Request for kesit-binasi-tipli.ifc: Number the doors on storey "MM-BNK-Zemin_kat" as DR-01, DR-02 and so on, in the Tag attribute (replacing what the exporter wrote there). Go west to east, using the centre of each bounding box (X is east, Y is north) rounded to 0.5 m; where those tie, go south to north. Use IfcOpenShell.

First a look at what the model holds.

```python
import ifcopenshell
import ifcopenshell.util.element
import ifcopenshell.util.placement

model = ifcopenshell.open("kesit-binasi-tipli.ifc")
print(model.schema)
storey = next(s for s in model.by_type("IfcBuildingStorey") if s.Name == "MM-BNK-Zemin_kat")
doors = [e for e in ifcopenshell.util.element.get_decomposition(storey) if e.is_a("IfcDoor")]
for e in sorted(doors, key=lambda e: e.id()):
    origin = ifcopenshell.util.placement.get_local_placement(e.ObjectPlacement)[:3, 3]
    print(e.id(), e.Tag, e.Name, origin.round(2) + 0.0, sep=" | ")
```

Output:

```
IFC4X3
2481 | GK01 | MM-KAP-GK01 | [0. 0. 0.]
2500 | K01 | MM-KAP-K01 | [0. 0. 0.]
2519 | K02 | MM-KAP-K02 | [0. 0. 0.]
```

```python
import ifcopenshell
import ifcopenshell.geom
import ifcopenshell.util.element
import ifcopenshell.util.shape

model = ifcopenshell.open("kesit-binasi-tipli.ifc")
settings = ifcopenshell.geom.settings()
settings.set("use-world-coords", True)


def centre(element):
    shape = ifcopenshell.geom.create_shape(settings, element)
    return ifcopenshell.util.shape.get_bbox_centroid(shape.geometry)


storey = next(s for s in model.by_type("IfcBuildingStorey") if s.Name == "MM-BNK-Zemin_kat")
doors = [e for e in ifcopenshell.util.element.get_decomposition(storey) if e.is_a("IfcDoor")]

# Insertion points can sit at a corner or the storey origin, so sort by the geometry (in metres).
centres = {e: centre(e) for e in doors}
doors.sort(key=lambda e: (round(centres[e][0] / 0.5), centres[e][1]))

for i, e in enumerate(doors, start=1):
    number = f"DR-{i:02d}"
    e.Tag = number
    print(e.id(), number)

model.write("kesit-binasi-tipli_edited.ifc")
```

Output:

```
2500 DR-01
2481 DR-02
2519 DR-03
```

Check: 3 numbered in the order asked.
